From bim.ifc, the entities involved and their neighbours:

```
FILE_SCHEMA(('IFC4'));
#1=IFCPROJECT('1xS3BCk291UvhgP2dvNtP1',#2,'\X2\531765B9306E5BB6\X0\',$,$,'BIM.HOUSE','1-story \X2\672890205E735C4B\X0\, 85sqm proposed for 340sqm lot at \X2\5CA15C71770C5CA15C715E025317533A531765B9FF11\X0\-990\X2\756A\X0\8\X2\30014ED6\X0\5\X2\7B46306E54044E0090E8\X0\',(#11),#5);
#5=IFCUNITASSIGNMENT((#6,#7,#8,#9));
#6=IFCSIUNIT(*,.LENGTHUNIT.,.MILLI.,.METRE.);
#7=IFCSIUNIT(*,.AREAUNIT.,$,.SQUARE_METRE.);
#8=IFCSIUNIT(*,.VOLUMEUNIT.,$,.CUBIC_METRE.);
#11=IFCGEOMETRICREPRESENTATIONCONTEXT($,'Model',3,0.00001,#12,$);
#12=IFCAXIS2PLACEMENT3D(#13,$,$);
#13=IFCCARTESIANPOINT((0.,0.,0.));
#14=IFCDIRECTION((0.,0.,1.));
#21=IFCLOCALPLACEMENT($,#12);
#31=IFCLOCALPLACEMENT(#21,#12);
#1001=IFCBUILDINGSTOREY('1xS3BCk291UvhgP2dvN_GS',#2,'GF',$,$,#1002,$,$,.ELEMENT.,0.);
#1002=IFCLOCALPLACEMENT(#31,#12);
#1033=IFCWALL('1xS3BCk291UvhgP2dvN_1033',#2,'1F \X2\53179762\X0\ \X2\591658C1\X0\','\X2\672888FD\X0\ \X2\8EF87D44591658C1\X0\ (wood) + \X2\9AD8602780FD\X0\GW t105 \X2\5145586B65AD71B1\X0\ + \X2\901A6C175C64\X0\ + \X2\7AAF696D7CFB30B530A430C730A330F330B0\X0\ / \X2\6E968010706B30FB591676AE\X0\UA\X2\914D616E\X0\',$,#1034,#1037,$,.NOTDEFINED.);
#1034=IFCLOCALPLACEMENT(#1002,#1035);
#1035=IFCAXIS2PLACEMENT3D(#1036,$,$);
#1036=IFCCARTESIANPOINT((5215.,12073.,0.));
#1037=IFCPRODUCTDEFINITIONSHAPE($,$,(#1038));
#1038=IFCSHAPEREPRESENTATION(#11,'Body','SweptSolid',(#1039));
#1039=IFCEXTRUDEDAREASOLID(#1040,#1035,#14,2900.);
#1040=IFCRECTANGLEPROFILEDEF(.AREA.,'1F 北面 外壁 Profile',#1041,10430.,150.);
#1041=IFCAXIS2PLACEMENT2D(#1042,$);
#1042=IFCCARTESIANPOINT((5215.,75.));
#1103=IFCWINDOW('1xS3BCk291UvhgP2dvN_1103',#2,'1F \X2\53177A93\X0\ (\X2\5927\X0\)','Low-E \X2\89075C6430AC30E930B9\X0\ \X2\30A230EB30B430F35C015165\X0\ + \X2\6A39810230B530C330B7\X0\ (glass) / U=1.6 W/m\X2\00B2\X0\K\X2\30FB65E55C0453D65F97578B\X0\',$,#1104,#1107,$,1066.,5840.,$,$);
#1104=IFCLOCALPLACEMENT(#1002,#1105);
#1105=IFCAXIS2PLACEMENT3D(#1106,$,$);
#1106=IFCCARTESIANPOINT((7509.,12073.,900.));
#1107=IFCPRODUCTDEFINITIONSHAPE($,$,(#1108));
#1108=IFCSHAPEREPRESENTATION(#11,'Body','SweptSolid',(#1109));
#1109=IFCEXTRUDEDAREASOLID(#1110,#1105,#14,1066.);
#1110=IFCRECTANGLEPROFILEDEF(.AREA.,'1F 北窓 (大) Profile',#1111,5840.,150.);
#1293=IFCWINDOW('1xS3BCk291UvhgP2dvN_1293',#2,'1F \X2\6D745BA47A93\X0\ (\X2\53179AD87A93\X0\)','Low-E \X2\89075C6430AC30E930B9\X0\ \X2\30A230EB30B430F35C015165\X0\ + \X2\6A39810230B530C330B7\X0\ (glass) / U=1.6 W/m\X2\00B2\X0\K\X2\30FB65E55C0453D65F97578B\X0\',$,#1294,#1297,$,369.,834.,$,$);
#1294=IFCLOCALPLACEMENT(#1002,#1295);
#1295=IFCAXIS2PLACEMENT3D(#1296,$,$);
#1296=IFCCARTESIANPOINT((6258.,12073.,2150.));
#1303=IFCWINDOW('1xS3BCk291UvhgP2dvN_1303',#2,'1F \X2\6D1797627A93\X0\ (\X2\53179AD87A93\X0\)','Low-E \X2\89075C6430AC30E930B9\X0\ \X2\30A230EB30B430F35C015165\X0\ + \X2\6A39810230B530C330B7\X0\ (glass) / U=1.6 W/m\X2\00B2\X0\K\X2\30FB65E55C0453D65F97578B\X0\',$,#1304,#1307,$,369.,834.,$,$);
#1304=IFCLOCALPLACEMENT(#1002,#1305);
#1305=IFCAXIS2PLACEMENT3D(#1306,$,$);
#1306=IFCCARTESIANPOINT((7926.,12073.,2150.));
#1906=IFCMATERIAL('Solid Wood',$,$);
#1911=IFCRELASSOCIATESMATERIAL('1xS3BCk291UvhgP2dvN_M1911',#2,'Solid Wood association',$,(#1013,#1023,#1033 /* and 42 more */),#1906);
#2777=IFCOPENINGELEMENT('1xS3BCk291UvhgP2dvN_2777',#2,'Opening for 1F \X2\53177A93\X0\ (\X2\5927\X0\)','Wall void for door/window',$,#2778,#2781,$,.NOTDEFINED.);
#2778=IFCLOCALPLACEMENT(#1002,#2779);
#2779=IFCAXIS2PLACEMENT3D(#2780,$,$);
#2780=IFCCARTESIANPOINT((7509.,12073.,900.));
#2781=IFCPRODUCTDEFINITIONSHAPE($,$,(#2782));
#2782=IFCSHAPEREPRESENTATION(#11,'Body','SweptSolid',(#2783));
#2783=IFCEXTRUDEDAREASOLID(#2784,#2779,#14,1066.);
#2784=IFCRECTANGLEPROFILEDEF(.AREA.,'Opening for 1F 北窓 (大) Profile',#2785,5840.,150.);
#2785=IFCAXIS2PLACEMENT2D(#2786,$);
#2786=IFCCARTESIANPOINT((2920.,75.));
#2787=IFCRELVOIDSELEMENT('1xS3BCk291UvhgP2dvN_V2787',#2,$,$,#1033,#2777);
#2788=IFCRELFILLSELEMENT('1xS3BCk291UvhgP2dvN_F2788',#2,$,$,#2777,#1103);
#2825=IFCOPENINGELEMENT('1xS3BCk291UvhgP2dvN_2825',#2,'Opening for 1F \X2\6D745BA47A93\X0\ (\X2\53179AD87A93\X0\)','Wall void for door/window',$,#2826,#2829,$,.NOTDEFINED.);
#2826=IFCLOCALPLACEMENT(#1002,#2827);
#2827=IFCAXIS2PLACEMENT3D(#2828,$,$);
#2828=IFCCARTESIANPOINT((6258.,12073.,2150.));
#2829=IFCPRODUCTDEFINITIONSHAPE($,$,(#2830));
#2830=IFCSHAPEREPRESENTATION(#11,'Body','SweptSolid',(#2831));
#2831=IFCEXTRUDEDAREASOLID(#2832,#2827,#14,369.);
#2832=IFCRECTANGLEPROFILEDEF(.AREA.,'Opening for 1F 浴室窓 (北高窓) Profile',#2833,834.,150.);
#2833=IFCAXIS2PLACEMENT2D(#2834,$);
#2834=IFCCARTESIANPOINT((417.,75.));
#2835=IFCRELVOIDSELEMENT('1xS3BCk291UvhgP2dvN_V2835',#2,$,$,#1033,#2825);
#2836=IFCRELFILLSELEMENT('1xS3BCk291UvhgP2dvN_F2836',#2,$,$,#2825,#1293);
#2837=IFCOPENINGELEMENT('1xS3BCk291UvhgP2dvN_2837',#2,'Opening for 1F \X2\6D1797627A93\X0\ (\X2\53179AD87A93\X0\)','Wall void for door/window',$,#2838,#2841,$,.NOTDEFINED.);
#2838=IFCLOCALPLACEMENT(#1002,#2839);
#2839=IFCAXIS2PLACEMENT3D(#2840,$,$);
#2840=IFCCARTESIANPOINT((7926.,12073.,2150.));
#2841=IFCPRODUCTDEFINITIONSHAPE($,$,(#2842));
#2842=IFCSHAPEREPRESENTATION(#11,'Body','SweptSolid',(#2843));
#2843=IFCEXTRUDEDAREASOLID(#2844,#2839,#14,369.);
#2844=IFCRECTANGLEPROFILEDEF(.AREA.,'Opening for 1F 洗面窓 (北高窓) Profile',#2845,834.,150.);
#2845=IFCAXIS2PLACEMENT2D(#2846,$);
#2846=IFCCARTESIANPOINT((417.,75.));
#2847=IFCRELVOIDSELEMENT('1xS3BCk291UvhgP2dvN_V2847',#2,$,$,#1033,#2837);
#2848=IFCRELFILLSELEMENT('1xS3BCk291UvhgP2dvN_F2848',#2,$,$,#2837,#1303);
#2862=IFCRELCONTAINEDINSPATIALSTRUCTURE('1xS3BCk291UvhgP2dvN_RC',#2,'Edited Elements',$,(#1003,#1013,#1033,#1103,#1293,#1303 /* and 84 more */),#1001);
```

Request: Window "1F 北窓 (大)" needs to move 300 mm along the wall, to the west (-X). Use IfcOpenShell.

```python
import ifcopenshell
import ifcopenshell.api.geometry
import ifcopenshell.util.placement
import ifcopenshell.util.unit

model = ifcopenshell.open("bim.ifc")
unit_scale = ifcopenshell.util.unit.calculate_unit_scale(model)

window = model.by_id(1103)
opening = window.FillsVoids[0].RelatingOpeningElement
wall = opening.VoidsElements[0].RelatingBuildingElement

wall_matrix = ifcopenshell.util.placement.get_local_placement(wall.ObjectPlacement)
shift = wall_matrix[:3, 0] * -0.3 / unit_scale
before = ifcopenshell.util.placement.get_local_placement(window.ObjectPlacement)[:3, 3].copy()

# The window is not placed relative to its opening, so move both.
for product in (opening, window):
    matrix = ifcopenshell.util.placement.get_local_placement(product.ObjectPlacement)
    matrix[:3, 3] += shift
    ifcopenshell.api.geometry.edit_object_placement(model, product=product, matrix=matrix, is_si=False)

after = ifcopenshell.util.placement.get_local_placement(window.ObjectPlacement)[:3, 3]
print("window moved by", (after - before).round(3) + 0.0)

model.write("bim_updated.ifc")
```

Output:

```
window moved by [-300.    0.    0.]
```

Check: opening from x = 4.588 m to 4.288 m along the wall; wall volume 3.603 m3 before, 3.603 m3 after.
